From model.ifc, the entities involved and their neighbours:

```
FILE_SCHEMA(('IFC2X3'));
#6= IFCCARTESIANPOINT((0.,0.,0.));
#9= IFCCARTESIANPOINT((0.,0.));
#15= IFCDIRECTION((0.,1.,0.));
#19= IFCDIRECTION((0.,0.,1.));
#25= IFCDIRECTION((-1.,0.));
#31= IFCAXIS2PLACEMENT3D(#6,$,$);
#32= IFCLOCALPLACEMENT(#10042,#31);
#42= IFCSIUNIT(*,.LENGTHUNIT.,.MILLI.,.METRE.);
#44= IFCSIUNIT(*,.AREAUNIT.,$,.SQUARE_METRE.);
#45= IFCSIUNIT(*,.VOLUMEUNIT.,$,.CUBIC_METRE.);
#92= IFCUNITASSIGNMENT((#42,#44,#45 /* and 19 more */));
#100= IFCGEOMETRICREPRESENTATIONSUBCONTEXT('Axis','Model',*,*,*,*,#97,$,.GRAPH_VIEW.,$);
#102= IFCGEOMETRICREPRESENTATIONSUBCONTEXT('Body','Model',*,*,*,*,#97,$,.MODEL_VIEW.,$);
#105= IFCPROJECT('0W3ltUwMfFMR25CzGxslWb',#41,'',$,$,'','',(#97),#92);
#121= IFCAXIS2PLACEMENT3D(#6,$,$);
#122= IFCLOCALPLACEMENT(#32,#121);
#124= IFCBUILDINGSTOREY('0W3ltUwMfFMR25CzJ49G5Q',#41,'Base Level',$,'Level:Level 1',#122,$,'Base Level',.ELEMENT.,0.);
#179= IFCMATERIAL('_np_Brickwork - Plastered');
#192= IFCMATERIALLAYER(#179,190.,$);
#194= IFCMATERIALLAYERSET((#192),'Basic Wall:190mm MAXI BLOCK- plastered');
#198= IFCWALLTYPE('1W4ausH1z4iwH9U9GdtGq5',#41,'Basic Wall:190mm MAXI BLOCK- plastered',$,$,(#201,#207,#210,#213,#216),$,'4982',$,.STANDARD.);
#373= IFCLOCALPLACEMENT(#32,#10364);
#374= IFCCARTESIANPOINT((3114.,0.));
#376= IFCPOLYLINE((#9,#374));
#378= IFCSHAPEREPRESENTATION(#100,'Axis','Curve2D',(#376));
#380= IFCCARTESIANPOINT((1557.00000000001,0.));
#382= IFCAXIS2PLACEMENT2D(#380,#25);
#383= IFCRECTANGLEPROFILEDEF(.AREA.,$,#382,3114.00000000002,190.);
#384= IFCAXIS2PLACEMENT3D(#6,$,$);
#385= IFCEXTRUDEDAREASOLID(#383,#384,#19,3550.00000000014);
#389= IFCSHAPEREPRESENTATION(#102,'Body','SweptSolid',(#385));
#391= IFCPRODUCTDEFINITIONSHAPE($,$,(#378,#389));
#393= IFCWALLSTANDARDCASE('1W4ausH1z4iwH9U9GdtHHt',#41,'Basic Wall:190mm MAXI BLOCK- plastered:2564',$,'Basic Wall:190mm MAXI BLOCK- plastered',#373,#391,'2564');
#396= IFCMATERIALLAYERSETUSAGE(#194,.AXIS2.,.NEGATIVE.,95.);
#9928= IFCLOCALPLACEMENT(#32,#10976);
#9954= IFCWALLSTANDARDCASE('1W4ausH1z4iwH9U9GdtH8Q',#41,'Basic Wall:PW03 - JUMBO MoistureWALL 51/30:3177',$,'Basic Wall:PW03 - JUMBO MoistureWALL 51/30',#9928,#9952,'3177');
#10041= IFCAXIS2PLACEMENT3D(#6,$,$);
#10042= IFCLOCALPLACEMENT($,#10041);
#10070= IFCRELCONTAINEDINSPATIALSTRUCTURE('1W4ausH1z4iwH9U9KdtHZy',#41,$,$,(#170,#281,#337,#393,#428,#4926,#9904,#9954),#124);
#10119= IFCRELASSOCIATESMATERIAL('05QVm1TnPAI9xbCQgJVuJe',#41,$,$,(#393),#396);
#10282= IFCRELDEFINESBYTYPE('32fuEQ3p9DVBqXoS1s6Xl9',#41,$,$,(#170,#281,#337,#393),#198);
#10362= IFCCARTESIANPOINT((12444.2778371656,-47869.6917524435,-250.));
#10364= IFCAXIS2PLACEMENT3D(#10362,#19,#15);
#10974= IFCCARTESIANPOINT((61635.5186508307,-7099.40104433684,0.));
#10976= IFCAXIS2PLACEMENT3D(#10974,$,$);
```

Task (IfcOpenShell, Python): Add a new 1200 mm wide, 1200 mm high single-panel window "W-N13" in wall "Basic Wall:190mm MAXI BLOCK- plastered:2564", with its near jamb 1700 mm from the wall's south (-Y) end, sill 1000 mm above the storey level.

```python
import numpy as np
import ifcopenshell
import ifcopenshell.api.feature
import ifcopenshell.api.geometry
import ifcopenshell.api.root
import ifcopenshell.api.spatial
import ifcopenshell.api.type
import ifcopenshell.geom
import ifcopenshell.util.element
import ifcopenshell.util.placement
import ifcopenshell.util.representation
import ifcopenshell.util.shape
import ifcopenshell.util.unit

model = ifcopenshell.open("model.ifc")
unit_scale = ifcopenshell.util.unit.calculate_unit_scale(model)
settings = ifcopenshell.geom.settings()


def volume(element):
    """Net volume in cubic metres, openings subtracted."""
    shape = ifcopenshell.geom.create_shape(settings, element)
    return ifcopenshell.util.shape.get_volume(shape.geometry)


wall = model.by_id(393)
storey = ifcopenshell.util.element.get_container(wall, ifc_class="IfcBuildingStorey")
context = ifcopenshell.util.representation.get_context(model, "Model", "Body", "MODEL_VIEW")
before = volume(wall)

width, height, from_end, sill = 1.2, 1.2, 1.7, 1  # metres

# The wall runs along its own X axis, and the end named is its -X end.
wall_shape = ifcopenshell.geom.create_shape(settings, wall)
x, y, z = ifcopenshell.util.shape.get_vertices(wall_shape.geometry).T
start = x.min() + from_end
face, thickness = float(y.min()), float(y.max() - y.min())
wall_matrix = ifcopenshell.util.placement.get_local_placement(wall.ObjectPlacement)
level = ifcopenshell.util.placement.get_local_placement(storey.ObjectPlacement)[2, 3]


def in_wall(x, y):
    """Placement at x, y metres in the wall's axes, at sill height."""
    matrix = wall_matrix.copy()
    matrix[:, 3] = wall_matrix @ np.array([x / unit_scale, y / unit_scale, 0.0, 1.0])
    matrix[2, 3] = level + sill / unit_scale
    return matrix


# Opening: a box that overshoots both wall faces by 50 mm.
opening = ifcopenshell.api.root.create_entity(model, ifc_class="IfcOpeningElement")
box = ifcopenshell.api.geometry.add_wall_representation(
    model, context=context, length=width, height=height, thickness=thickness + 0.1
)
ifcopenshell.api.geometry.assign_representation(model, product=opening, representation=box)
ifcopenshell.api.geometry.edit_object_placement(model, product=opening, matrix=in_wall(start, face - 0.05), is_si=False)
ifcopenshell.api.feature.add_feature(model, feature=opening, element=wall)

window = ifcopenshell.api.root.create_entity(model, ifc_class="IfcWindow", name="W-N13")
window.OverallWidth, window.OverallHeight = width / unit_scale, height / unit_scale
body = ifcopenshell.api.geometry.add_window_representation(
    model,
    context=context,
    overall_width=window.OverallWidth,
    overall_height=window.OverallHeight,
    partition_type="SINGLE_PANEL",
)
ifcopenshell.api.geometry.assign_representation(model, product=window, representation=body)
ifcopenshell.api.spatial.assign_container(model, products=[window], relating_structure=storey)
fills = ifcopenshell.api.feature.add_filling(model, opening=opening, element=window)
fills.OwnerHistory = window.OwnerHistory  # required in IFC2X3

# IFC2X3 keeps the operation on the window style.
style = ifcopenshell.api.root.create_entity(model, ifc_class="IfcWindowStyle", name="W-N13")
style.OperationType, style.ConstructionType = "SINGLE_PANEL", "NOTDEFINED"
style.ParameterTakesPrecedence = style.Sizeable = False
ifcopenshell.api.type.assign_type(model, related_objects=[window], relating_type=style)

# Centre the window in the wall's thickness.
ifcopenshell.api.geometry.edit_object_placement(model, product=window, matrix=in_wall(start, face), is_si=False)
window_shape = ifcopenshell.geom.create_shape(settings, window)
depth = ifcopenshell.util.shape.get_vertices(window_shape.geometry)[:, 1]
offset = face + thickness / 2 - (depth.min() + depth.max()) / 2
ifcopenshell.api.geometry.edit_object_placement(model, product=window, matrix=in_wall(start, offset), is_si=False)

after = volume(wall)

print(f"wall volume {before:.3f} -> {after:.3f} m3")

model.write("model_edited.ifc")
```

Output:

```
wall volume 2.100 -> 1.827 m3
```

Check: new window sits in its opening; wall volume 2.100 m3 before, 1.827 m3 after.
